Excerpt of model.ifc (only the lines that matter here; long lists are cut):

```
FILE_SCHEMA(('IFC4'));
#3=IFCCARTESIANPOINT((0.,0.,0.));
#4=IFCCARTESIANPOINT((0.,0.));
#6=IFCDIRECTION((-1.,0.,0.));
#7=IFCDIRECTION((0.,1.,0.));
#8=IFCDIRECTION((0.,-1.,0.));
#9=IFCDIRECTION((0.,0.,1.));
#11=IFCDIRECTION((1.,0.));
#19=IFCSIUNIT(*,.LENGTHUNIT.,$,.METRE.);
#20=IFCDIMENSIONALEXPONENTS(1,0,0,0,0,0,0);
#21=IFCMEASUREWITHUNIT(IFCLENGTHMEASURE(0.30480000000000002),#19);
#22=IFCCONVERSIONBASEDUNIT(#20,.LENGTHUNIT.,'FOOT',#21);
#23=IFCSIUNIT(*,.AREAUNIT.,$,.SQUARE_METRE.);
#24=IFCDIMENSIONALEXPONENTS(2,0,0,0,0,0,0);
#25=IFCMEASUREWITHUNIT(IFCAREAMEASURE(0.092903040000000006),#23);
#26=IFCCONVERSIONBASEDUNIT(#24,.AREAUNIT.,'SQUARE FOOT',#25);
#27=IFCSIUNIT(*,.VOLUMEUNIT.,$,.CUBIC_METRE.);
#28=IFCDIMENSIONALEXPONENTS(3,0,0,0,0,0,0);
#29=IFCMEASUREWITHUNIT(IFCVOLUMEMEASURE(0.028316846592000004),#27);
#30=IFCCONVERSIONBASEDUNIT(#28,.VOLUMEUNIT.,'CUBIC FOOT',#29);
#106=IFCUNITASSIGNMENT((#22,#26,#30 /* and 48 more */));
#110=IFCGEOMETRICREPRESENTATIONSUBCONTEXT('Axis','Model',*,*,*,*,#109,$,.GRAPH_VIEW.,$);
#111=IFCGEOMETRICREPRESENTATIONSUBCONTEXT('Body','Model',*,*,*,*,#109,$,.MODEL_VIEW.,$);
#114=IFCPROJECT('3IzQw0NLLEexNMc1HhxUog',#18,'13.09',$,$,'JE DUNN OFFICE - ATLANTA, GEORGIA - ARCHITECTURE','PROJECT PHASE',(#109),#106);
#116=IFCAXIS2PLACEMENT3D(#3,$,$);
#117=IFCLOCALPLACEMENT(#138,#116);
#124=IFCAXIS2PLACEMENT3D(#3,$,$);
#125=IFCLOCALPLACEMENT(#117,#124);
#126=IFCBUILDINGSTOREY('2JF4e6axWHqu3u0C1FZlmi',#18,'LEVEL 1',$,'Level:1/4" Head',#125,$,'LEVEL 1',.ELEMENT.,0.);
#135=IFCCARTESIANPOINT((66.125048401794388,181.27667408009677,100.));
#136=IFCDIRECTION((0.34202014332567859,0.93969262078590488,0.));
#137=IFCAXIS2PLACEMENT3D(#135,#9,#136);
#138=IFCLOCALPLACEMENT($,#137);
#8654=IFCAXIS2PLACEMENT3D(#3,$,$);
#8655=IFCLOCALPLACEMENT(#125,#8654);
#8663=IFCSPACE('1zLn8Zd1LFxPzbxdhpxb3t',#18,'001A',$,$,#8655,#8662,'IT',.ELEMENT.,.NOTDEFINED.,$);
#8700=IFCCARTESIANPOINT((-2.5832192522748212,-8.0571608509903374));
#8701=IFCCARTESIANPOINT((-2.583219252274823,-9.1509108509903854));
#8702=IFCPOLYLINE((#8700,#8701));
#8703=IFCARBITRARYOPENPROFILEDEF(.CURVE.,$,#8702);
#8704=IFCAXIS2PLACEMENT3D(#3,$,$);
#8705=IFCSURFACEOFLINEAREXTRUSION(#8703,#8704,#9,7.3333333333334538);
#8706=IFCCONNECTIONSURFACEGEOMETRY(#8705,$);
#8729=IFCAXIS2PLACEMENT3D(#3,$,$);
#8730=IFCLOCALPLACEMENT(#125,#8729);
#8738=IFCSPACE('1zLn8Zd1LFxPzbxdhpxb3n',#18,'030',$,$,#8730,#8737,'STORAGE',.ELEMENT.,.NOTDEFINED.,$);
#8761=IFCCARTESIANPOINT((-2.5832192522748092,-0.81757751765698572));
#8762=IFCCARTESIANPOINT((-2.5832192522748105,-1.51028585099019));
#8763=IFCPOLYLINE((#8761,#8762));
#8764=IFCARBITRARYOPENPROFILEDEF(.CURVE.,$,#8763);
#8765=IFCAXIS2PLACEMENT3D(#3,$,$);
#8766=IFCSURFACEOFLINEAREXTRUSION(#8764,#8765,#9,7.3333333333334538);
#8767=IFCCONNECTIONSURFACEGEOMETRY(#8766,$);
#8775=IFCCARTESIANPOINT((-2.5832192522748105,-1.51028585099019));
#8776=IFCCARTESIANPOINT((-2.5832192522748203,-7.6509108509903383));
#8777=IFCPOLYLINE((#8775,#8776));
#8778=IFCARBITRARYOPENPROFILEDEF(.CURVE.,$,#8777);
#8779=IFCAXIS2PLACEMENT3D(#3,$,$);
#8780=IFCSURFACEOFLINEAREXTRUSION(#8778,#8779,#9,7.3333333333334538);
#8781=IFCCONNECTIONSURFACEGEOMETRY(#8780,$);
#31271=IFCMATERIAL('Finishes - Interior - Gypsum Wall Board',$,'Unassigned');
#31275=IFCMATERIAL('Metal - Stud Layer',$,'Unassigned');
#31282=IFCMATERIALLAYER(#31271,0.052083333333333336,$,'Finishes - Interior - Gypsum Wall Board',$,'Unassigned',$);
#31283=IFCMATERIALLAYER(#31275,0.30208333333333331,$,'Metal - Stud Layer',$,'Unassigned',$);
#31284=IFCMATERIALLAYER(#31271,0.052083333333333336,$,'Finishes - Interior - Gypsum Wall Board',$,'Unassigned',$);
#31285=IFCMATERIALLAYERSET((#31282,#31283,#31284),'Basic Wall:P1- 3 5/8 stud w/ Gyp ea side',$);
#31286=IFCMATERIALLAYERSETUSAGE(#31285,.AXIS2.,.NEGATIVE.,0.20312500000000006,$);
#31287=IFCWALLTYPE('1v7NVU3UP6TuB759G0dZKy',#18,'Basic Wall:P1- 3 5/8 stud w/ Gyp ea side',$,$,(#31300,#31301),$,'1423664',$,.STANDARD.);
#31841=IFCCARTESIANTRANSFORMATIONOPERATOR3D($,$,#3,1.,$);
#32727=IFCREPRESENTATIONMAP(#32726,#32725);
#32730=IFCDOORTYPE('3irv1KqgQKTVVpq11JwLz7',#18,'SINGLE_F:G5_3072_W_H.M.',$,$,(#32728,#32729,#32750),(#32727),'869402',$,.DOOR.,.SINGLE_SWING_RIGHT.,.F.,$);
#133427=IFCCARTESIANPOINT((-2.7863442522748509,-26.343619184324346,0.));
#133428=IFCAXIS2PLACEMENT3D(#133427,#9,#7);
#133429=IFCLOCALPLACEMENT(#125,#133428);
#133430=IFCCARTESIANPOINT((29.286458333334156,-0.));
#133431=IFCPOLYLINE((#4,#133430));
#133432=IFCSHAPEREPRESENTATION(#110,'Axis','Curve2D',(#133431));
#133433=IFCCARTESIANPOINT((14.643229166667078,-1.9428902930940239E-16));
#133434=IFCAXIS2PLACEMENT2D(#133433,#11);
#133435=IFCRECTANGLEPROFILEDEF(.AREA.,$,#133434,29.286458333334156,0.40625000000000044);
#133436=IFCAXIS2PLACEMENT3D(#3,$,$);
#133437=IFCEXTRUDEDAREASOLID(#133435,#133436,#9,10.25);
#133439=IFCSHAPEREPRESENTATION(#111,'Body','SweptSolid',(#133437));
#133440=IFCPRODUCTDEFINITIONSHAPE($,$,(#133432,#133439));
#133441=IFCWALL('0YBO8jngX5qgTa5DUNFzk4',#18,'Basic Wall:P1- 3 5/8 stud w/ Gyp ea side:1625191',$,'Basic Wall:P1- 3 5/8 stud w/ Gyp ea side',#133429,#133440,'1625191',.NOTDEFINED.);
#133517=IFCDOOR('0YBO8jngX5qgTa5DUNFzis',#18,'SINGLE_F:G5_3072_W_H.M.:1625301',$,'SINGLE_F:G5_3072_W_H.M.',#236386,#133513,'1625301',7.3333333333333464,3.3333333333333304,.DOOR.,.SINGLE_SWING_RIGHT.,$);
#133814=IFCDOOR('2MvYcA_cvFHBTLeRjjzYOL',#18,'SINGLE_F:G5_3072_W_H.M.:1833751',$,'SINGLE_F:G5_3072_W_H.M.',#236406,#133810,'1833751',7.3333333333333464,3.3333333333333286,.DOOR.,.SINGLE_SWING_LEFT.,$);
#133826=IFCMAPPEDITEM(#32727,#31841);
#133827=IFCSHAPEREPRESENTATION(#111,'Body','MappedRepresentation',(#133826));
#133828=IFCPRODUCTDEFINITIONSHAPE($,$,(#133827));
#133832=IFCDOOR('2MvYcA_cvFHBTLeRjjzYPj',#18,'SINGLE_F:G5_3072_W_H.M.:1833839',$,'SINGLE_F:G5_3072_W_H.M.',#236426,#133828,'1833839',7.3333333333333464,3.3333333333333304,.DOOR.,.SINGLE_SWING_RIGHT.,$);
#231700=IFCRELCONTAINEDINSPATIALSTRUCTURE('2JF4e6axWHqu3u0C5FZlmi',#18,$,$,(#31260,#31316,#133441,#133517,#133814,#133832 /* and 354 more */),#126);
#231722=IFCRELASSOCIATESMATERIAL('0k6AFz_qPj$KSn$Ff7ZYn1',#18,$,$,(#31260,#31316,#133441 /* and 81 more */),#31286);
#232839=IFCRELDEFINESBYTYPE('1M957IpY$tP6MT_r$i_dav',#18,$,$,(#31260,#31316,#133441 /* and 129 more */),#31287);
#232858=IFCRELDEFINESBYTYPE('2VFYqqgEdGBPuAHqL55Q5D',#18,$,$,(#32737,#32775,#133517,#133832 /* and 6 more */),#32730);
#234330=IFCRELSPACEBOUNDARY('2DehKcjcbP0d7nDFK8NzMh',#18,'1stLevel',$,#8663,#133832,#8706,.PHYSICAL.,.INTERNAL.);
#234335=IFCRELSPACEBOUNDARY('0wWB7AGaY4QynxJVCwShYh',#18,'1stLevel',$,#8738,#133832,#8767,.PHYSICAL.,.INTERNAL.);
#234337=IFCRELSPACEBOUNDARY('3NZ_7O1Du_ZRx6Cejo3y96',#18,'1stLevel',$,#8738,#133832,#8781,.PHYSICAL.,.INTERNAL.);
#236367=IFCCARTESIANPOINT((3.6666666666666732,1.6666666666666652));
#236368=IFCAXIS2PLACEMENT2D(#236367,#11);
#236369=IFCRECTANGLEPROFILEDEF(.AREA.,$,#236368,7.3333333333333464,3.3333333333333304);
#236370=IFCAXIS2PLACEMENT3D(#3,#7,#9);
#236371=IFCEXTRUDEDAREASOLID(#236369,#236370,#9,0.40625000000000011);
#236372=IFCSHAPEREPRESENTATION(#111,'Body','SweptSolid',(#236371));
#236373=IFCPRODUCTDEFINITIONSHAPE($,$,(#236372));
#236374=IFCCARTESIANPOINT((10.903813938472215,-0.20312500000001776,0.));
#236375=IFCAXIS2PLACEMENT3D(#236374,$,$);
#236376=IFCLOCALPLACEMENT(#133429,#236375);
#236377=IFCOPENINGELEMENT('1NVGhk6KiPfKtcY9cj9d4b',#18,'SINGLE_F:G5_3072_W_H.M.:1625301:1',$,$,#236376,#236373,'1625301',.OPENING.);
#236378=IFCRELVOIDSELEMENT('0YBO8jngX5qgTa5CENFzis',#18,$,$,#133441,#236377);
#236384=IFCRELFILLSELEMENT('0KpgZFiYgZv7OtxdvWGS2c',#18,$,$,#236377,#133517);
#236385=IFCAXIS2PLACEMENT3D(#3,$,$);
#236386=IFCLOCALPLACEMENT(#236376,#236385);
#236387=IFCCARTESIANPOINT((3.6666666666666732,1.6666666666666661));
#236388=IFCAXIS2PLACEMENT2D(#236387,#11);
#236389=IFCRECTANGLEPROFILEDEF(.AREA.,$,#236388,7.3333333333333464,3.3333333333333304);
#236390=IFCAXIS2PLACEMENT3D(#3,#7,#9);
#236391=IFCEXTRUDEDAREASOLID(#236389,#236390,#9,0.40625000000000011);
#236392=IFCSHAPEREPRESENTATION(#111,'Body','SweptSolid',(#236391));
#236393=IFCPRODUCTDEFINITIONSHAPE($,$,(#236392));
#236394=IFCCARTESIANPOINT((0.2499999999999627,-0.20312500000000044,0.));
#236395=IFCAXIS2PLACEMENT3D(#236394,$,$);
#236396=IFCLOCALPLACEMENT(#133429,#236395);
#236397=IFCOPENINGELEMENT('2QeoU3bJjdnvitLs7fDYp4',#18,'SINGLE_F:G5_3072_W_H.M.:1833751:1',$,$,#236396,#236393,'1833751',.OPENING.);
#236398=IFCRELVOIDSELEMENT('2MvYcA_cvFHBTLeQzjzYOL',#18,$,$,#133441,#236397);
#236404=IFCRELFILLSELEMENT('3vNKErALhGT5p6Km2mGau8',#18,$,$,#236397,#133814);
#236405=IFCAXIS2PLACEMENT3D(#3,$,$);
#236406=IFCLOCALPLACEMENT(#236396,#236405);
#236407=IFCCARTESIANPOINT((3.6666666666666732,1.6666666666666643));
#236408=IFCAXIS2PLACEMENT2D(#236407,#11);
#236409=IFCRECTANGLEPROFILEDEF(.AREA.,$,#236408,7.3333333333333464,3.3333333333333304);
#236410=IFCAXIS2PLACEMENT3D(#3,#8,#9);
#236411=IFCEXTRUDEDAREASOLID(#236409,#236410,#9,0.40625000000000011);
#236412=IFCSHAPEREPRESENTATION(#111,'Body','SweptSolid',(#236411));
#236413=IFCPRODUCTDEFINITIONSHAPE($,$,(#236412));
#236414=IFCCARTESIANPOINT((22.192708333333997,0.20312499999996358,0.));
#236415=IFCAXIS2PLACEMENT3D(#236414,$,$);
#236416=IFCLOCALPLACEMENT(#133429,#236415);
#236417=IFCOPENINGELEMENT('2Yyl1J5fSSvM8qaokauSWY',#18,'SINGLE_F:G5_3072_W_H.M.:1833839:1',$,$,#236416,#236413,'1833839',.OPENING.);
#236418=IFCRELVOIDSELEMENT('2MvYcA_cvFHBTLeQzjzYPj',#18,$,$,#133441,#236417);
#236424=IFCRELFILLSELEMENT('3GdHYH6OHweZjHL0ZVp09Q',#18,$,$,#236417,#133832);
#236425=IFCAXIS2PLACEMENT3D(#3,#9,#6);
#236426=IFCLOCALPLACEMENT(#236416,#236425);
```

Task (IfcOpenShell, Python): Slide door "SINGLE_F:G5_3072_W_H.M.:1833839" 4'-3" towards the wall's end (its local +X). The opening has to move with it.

```python
import numpy as np
import ifcopenshell
import ifcopenshell.api.geometry
import ifcopenshell.util.placement
import ifcopenshell.util.unit

model = ifcopenshell.open("model.ifc")
unit_scale = ifcopenshell.util.unit.calculate_unit_scale(model)

door = model.by_guid("2MvYcA_cvFHBTLeRjjzYPj")
opening = door.FillsVoids[0].RelatingOpeningElement
wall = opening.VoidsElements[0].RelatingBuildingElement

wall_matrix = ifcopenshell.util.placement.get_local_placement(wall.ObjectPlacement)
shift = wall_matrix[:3, 0] * 51 * 0.0254 / unit_scale
before = ifcopenshell.util.placement.get_local_placement(door.ObjectPlacement)[:3, 3].copy()

# The door is placed relative to its opening, so it follows when the opening moves.
matrix = ifcopenshell.util.placement.get_local_placement(opening.ObjectPlacement)
matrix[:3, 3] += shift
ifcopenshell.api.geometry.edit_object_placement(
    model, product=opening, matrix=matrix, is_si=False, should_transform_children=True
)

# Space boundary surfaces are stored in each space's coordinates; move them too.
for rel in door.ProvidesBoundaries:
    if not rel.ConnectionGeometry:
        continue
    surface = rel.ConnectionGeometry.SurfaceOnRelatingElement
    space_matrix = ifcopenshell.util.placement.get_local_placement(rel.RelatingSpace.ObjectPlacement)
    point = np.array(surface.Position.Location.Coordinates) + space_matrix[:3, :3].T @ shift
    surface.Position = model.createIfcAxis2Placement3D(
        model.createIfcCartesianPoint(point.tolist()), surface.Position.Axis, surface.Position.RefDirection
    )

after = ifcopenshell.util.placement.get_local_placement(door.ObjectPlacement)[:3, 3]
print("door moved by", (after - before).round(3) + 0.0)

model.write("model-out.ifc")
```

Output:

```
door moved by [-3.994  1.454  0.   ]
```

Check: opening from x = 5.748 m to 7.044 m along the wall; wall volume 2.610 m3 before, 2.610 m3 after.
